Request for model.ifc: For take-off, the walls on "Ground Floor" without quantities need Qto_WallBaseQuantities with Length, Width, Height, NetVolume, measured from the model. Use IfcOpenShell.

First a look at what the model holds.

```python
import ifcopenshell
import ifcopenshell.util.element
import ifcopenshell.util.unit

model = ifcopenshell.open("model.ifc")
print(model.schema)
for unit_type in ("LENGTHUNIT", "AREAUNIT", "VOLUMEUNIT"):
    print(unit_type, ifcopenshell.util.unit.calculate_unit_scale(model, unit_type))
storey = next(s for s in model.by_type("IfcBuildingStorey") if s.Name == "Ground Floor")
walls = [e for e in ifcopenshell.util.element.get_decomposition(storey) if e.is_a("IfcWall")]
for e in sorted(walls, key=lambda e: e.id()):
    print(e.id(), e.is_a(), e.Name, list(ifcopenshell.util.element.get_psets(e, qtos_only=True)), sep=" | ")
```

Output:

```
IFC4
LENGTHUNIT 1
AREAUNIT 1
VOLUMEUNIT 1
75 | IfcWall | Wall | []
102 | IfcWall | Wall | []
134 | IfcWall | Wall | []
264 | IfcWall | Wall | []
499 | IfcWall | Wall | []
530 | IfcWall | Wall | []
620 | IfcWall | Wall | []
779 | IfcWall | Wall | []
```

```python
import ifcopenshell
import ifcopenshell.api.pset
import ifcopenshell.geom
import ifcopenshell.util.element
import ifcopenshell.util.shape
import ifcopenshell.util.unit

model = ifcopenshell.open("model.ifc")
unit_scale = ifcopenshell.util.unit.calculate_unit_scale(model)
volume_scale = ifcopenshell.util.unit.calculate_unit_scale(model, "VOLUMEUNIT")
settings = ifcopenshell.geom.settings()

storey = next(s for s in model.by_type("IfcBuildingStorey") if s.Name == "Ground Floor")
walls = [e for e in ifcopenshell.util.element.get_decomposition(storey) if e.is_a("IfcWall")]

for e in sorted(walls, key=lambda e: e.id()):
    if ifcopenshell.util.element.get_psets(e, qtos_only=True, should_inherit=False):
        continue
    # Geometry comes back in metres, in the element's own axes.
    shape = ifcopenshell.geom.create_shape(settings, e)
    values = {
        "Length": ifcopenshell.util.shape.get_x(shape.geometry) / unit_scale,
        "Width": ifcopenshell.util.shape.get_y(shape.geometry) / unit_scale,
        "Height": ifcopenshell.util.shape.get_z(shape.geometry) / unit_scale,
        "NetVolume": ifcopenshell.util.shape.get_volume(shape.geometry) / volume_scale,
    }
    qto = ifcopenshell.api.pset.add_qto(model, product=e, name="Qto_WallBaseQuantities")
    ifcopenshell.api.pset.edit_qto(model, qto=qto, properties=values)
    print(e.id(), {k: round(v, 3) for k, v in values.items()})

model.write("model_v2.ifc")
```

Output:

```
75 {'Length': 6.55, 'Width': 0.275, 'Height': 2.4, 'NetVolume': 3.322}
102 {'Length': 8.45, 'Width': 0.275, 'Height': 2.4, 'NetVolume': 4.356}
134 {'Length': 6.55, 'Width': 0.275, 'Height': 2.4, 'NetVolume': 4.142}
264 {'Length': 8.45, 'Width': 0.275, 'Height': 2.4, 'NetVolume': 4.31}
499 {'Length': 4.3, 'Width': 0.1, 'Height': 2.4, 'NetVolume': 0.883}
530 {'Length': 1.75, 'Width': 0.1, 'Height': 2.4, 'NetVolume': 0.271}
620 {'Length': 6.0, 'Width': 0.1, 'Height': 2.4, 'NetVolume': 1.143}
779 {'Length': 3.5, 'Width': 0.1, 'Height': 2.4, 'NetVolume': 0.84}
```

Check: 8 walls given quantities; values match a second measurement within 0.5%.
